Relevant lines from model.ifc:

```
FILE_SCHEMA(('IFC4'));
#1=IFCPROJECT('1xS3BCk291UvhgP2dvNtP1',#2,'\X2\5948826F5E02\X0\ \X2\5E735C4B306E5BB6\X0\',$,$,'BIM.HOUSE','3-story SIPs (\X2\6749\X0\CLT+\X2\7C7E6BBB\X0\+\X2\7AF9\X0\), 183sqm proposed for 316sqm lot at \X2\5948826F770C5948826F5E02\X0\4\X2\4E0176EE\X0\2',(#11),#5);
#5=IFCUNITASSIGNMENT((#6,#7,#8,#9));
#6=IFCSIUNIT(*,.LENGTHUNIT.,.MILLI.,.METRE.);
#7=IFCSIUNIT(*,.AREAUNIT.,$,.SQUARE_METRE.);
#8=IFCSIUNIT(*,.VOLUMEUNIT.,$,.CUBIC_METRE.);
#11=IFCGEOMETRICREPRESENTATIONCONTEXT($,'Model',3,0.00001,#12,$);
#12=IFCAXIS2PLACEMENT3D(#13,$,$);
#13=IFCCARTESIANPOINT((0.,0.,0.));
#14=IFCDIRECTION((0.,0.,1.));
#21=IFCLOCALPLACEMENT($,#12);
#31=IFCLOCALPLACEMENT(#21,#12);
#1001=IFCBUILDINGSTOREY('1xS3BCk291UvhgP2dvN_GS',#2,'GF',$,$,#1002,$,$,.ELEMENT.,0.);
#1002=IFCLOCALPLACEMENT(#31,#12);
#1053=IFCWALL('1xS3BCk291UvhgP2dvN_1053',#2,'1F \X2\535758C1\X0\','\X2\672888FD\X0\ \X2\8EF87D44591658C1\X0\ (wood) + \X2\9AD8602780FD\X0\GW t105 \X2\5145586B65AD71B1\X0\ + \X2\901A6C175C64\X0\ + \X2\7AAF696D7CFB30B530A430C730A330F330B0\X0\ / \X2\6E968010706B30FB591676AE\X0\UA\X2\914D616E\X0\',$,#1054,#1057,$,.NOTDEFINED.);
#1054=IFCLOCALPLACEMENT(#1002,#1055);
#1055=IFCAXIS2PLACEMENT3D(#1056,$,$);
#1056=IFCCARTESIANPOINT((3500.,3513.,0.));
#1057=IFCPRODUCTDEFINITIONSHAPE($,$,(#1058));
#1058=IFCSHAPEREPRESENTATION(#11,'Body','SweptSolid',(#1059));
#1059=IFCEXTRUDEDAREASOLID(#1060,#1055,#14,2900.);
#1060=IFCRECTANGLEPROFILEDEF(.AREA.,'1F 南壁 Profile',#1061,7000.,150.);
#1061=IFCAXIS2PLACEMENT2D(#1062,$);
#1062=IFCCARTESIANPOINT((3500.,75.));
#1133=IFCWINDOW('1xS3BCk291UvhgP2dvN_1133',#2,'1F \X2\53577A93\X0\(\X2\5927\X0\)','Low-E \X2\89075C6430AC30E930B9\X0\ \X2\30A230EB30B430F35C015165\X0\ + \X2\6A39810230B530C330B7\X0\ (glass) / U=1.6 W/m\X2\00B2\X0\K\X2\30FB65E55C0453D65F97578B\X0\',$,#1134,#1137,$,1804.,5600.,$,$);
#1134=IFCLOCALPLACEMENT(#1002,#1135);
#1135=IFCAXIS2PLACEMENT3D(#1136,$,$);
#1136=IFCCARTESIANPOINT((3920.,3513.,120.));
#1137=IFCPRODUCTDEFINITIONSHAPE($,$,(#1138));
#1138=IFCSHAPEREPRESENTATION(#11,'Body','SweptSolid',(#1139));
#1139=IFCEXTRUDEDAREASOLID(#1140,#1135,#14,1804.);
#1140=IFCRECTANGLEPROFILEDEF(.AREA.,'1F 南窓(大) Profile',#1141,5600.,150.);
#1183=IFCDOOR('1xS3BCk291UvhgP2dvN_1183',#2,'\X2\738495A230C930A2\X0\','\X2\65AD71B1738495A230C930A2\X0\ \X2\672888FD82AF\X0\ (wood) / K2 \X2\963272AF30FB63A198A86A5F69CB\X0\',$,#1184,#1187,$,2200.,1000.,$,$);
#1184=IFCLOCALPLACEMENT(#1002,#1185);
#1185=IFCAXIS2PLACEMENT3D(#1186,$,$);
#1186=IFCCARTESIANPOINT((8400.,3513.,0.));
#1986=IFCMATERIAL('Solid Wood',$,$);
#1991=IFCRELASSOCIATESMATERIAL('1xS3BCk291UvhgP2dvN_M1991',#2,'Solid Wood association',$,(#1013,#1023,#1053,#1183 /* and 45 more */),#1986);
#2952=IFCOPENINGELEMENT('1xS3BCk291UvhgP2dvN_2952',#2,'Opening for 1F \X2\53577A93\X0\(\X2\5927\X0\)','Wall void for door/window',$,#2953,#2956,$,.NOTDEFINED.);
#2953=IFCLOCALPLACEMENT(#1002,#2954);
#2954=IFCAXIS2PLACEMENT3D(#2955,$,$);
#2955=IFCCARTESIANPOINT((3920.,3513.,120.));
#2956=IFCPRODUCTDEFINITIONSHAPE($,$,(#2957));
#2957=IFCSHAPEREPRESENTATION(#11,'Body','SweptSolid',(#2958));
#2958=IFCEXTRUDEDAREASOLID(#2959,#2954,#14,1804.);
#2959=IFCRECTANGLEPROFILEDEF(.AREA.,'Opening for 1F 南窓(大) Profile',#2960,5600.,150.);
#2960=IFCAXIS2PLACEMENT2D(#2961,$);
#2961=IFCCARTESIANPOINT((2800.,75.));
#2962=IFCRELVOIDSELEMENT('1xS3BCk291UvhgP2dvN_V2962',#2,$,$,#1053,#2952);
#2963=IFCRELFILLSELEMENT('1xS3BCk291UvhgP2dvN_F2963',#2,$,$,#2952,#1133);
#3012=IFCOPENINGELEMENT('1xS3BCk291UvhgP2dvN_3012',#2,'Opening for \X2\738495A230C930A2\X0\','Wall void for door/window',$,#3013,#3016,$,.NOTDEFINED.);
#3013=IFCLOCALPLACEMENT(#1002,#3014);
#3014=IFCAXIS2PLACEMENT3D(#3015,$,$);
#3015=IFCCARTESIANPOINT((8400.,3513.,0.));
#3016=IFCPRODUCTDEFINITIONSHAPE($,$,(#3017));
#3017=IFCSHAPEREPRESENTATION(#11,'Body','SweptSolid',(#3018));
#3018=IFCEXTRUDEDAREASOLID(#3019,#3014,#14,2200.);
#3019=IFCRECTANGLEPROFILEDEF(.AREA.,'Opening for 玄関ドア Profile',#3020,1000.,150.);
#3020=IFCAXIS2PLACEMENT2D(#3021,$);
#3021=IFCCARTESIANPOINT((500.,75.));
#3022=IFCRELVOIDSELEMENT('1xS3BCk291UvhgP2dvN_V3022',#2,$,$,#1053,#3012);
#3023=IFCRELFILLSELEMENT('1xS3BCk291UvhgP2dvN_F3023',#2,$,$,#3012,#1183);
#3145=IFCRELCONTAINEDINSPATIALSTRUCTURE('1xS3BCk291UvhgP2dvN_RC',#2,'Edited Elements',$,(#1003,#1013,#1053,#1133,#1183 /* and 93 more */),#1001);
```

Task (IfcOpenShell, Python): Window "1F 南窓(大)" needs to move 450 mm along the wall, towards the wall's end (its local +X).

```python
import ifcopenshell
import ifcopenshell.api.geometry
import ifcopenshell.util.placement
import ifcopenshell.util.unit

model = ifcopenshell.open("model.ifc")
unit_scale = ifcopenshell.util.unit.calculate_unit_scale(model)

window = model.by_id(1133)
opening = window.FillsVoids[0].RelatingOpeningElement
wall = opening.VoidsElements[0].RelatingBuildingElement

wall_matrix = ifcopenshell.util.placement.get_local_placement(wall.ObjectPlacement)
shift = wall_matrix[:3, 0] * 0.45 / unit_scale
before = ifcopenshell.util.placement.get_local_placement(window.ObjectPlacement)[:3, 3].copy()

# The window is not placed relative to its opening, so move both.
for product in (opening, window):
    matrix = ifcopenshell.util.placement.get_local_placement(product.ObjectPlacement)
    matrix[:3, 3] += shift
    ifcopenshell.api.geometry.edit_object_placement(model, product=product, matrix=matrix, is_si=False)

after = ifcopenshell.util.placement.get_local_placement(window.ObjectPlacement)[:3, 3]
print("window moved by", (after - before).round(3) + 0.0)

model.write("model_edited.ifc")
```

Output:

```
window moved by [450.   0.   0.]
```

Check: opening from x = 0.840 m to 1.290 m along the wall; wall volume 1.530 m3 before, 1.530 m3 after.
